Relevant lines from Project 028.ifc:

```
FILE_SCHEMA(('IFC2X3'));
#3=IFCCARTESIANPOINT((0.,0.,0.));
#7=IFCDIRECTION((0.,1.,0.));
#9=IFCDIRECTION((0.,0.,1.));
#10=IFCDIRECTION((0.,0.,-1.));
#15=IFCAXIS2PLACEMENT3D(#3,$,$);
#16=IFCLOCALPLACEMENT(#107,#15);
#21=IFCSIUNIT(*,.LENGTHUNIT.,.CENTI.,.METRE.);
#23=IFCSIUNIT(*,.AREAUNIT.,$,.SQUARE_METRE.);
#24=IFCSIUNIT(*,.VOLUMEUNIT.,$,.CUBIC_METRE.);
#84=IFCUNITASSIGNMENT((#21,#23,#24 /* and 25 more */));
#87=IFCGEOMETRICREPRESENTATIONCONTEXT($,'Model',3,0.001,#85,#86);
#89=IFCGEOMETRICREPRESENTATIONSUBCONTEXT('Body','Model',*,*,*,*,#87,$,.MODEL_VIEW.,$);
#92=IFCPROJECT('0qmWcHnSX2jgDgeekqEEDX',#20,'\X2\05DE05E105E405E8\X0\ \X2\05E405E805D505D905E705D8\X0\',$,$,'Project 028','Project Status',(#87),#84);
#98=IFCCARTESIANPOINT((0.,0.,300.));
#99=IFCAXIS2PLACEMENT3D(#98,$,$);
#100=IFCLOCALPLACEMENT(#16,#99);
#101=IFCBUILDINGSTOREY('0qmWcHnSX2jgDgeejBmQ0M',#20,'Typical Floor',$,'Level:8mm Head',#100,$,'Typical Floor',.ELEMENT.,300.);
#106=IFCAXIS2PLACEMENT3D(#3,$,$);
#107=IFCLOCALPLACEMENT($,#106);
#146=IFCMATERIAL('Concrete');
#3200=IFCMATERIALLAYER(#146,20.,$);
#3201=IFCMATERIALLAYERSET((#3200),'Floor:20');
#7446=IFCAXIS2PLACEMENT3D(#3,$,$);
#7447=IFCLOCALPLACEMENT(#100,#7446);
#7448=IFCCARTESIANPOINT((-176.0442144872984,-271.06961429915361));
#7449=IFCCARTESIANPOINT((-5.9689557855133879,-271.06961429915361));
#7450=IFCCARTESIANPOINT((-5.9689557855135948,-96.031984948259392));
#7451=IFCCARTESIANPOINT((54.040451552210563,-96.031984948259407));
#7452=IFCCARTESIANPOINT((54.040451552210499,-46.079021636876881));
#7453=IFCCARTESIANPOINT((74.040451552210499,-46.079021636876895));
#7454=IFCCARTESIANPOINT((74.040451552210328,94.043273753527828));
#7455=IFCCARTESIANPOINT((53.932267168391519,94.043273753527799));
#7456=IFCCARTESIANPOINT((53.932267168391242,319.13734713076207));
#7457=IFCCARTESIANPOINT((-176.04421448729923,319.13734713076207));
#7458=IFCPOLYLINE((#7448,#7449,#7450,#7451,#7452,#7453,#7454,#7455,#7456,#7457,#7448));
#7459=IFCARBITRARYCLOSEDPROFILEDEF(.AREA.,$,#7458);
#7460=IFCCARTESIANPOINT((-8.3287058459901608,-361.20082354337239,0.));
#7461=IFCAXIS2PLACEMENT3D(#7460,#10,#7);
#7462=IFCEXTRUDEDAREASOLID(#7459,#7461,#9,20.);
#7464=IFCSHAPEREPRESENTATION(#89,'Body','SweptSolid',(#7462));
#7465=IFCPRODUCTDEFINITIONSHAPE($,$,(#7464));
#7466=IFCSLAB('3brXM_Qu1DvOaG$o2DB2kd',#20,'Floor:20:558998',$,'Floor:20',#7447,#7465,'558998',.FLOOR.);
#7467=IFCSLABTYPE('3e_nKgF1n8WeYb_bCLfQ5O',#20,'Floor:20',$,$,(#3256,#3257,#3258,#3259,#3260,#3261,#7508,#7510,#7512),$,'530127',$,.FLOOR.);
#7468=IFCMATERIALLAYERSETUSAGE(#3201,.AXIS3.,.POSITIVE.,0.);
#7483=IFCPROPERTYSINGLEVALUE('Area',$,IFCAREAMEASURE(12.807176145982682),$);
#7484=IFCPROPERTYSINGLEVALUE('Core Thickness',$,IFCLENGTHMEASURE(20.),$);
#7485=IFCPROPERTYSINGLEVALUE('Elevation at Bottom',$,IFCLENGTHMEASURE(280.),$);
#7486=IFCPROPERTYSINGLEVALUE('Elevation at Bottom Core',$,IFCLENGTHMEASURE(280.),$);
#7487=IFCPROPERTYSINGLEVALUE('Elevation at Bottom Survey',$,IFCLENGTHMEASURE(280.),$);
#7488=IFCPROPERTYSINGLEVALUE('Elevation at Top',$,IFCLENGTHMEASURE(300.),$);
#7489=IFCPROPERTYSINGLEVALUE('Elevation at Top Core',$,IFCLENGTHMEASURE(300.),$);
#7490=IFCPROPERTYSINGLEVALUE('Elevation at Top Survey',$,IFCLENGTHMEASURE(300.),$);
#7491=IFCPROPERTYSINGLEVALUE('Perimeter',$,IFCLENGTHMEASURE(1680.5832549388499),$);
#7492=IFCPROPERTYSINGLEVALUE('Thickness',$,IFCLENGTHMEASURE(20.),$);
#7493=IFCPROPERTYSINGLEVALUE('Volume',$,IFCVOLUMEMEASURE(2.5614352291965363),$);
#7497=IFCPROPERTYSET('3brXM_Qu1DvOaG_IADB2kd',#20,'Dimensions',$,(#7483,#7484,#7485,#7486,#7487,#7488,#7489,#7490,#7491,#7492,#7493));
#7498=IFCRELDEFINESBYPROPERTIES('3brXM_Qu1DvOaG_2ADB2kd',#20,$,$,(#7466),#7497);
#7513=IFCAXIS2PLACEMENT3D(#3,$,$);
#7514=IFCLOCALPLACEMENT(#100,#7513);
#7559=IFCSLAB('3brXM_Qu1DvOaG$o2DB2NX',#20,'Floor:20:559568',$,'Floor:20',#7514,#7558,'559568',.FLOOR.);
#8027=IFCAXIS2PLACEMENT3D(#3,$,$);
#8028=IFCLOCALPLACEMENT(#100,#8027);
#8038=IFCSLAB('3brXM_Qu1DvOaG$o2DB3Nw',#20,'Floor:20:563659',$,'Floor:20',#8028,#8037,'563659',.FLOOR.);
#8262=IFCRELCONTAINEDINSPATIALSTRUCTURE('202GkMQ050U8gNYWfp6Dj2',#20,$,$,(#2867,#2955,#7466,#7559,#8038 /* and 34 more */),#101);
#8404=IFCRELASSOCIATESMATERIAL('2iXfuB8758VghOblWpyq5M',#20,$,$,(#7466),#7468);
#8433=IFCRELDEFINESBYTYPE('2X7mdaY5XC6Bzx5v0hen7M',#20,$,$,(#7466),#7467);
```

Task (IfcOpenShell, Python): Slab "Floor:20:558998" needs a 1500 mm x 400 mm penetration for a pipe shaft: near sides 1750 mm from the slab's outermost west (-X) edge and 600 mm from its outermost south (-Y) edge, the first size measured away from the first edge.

```python
import numpy as np
import ifcopenshell
import ifcopenshell.api.feature
import ifcopenshell.api.geometry
import ifcopenshell.api.pset
import ifcopenshell.api.root
import ifcopenshell.geom
import ifcopenshell.util.element
import ifcopenshell.util.placement
import ifcopenshell.util.representation
import ifcopenshell.util.shape
import ifcopenshell.util.unit

model = ifcopenshell.open("Project 028.ifc")
unit_scale = ifcopenshell.util.unit.calculate_unit_scale(model)
area_scale = ifcopenshell.util.unit.calculate_unit_scale(model, "AREAUNIT")
volume_scale = ifcopenshell.util.unit.calculate_unit_scale(model, "VOLUMEUNIT")
settings = ifcopenshell.geom.settings()


def volume(element):
    """Net volume in cubic metres, openings subtracted."""
    shape = ifcopenshell.geom.create_shape(settings, element)
    return ifcopenshell.util.shape.get_volume(shape.geometry)


slab = model.by_guid("3brXM_Qu1DvOaG$o2DB2kd")
before = volume(slab)

# Extent in the slab's own axes, in metres. The edges named are its -X and -Y sides.
slab_shape = ifcopenshell.geom.create_shape(settings, slab)
vertices = ifcopenshell.util.shape.get_vertices(slab_shape.geometry)
x_min, y_min, bottom = vertices.min(axis=0)
top = vertices[:, 2].max()

opening = ifcopenshell.api.root.create_entity(model, ifc_class="IfcOpeningElement", name="Pipe shaft opening")
context = ifcopenshell.util.representation.get_context(model, "Model", "Body", "MODEL_VIEW")
width, depth = 1.5, 0.4
outline = [(0.0, 0.0), (width, 0.0), (width, depth), (0.0, depth), (0.0, 0.0)]
# Overshoot both faces by 50 mm so the cut is clean.
shape = ifcopenshell.api.geometry.add_slab_representation(
    model, context=context, depth=top - bottom + 0.1, polyline=outline
)
ifcopenshell.api.geometry.assign_representation(model, product=opening, representation=shape)

matrix = ifcopenshell.util.placement.get_local_placement(slab.ObjectPlacement)
matrix[:, 3] = matrix @ np.append(np.array([x_min + 1.75, y_min + 0.6, bottom - 0.05]) / unit_scale, 1.0)
ifcopenshell.api.geometry.edit_object_placement(model, product=opening, matrix=matrix, is_si=False)
ifcopenshell.api.feature.add_feature(model, feature=opening, element=slab)

after = volume(slab)

# Update the slab's stored quantities.
pset = model.by_id(ifcopenshell.util.element.get_pset(slab, "Dimensions", should_inherit=False)["id"])
ifcopenshell.api.pset.edit_pset(model, pset=pset, properties={
    "Area": model.create_entity("IfcAreaMeasure", after / (top - bottom) / area_scale),
    "Volume": model.create_entity("IfcVolumeMeasure", after / volume_scale),
})

print(f"slab volume {before:.3f} -> {after:.3f} m3")

model.write("Project 028_edited.ifc")
```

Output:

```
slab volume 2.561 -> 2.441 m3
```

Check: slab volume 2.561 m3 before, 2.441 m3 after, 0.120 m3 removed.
